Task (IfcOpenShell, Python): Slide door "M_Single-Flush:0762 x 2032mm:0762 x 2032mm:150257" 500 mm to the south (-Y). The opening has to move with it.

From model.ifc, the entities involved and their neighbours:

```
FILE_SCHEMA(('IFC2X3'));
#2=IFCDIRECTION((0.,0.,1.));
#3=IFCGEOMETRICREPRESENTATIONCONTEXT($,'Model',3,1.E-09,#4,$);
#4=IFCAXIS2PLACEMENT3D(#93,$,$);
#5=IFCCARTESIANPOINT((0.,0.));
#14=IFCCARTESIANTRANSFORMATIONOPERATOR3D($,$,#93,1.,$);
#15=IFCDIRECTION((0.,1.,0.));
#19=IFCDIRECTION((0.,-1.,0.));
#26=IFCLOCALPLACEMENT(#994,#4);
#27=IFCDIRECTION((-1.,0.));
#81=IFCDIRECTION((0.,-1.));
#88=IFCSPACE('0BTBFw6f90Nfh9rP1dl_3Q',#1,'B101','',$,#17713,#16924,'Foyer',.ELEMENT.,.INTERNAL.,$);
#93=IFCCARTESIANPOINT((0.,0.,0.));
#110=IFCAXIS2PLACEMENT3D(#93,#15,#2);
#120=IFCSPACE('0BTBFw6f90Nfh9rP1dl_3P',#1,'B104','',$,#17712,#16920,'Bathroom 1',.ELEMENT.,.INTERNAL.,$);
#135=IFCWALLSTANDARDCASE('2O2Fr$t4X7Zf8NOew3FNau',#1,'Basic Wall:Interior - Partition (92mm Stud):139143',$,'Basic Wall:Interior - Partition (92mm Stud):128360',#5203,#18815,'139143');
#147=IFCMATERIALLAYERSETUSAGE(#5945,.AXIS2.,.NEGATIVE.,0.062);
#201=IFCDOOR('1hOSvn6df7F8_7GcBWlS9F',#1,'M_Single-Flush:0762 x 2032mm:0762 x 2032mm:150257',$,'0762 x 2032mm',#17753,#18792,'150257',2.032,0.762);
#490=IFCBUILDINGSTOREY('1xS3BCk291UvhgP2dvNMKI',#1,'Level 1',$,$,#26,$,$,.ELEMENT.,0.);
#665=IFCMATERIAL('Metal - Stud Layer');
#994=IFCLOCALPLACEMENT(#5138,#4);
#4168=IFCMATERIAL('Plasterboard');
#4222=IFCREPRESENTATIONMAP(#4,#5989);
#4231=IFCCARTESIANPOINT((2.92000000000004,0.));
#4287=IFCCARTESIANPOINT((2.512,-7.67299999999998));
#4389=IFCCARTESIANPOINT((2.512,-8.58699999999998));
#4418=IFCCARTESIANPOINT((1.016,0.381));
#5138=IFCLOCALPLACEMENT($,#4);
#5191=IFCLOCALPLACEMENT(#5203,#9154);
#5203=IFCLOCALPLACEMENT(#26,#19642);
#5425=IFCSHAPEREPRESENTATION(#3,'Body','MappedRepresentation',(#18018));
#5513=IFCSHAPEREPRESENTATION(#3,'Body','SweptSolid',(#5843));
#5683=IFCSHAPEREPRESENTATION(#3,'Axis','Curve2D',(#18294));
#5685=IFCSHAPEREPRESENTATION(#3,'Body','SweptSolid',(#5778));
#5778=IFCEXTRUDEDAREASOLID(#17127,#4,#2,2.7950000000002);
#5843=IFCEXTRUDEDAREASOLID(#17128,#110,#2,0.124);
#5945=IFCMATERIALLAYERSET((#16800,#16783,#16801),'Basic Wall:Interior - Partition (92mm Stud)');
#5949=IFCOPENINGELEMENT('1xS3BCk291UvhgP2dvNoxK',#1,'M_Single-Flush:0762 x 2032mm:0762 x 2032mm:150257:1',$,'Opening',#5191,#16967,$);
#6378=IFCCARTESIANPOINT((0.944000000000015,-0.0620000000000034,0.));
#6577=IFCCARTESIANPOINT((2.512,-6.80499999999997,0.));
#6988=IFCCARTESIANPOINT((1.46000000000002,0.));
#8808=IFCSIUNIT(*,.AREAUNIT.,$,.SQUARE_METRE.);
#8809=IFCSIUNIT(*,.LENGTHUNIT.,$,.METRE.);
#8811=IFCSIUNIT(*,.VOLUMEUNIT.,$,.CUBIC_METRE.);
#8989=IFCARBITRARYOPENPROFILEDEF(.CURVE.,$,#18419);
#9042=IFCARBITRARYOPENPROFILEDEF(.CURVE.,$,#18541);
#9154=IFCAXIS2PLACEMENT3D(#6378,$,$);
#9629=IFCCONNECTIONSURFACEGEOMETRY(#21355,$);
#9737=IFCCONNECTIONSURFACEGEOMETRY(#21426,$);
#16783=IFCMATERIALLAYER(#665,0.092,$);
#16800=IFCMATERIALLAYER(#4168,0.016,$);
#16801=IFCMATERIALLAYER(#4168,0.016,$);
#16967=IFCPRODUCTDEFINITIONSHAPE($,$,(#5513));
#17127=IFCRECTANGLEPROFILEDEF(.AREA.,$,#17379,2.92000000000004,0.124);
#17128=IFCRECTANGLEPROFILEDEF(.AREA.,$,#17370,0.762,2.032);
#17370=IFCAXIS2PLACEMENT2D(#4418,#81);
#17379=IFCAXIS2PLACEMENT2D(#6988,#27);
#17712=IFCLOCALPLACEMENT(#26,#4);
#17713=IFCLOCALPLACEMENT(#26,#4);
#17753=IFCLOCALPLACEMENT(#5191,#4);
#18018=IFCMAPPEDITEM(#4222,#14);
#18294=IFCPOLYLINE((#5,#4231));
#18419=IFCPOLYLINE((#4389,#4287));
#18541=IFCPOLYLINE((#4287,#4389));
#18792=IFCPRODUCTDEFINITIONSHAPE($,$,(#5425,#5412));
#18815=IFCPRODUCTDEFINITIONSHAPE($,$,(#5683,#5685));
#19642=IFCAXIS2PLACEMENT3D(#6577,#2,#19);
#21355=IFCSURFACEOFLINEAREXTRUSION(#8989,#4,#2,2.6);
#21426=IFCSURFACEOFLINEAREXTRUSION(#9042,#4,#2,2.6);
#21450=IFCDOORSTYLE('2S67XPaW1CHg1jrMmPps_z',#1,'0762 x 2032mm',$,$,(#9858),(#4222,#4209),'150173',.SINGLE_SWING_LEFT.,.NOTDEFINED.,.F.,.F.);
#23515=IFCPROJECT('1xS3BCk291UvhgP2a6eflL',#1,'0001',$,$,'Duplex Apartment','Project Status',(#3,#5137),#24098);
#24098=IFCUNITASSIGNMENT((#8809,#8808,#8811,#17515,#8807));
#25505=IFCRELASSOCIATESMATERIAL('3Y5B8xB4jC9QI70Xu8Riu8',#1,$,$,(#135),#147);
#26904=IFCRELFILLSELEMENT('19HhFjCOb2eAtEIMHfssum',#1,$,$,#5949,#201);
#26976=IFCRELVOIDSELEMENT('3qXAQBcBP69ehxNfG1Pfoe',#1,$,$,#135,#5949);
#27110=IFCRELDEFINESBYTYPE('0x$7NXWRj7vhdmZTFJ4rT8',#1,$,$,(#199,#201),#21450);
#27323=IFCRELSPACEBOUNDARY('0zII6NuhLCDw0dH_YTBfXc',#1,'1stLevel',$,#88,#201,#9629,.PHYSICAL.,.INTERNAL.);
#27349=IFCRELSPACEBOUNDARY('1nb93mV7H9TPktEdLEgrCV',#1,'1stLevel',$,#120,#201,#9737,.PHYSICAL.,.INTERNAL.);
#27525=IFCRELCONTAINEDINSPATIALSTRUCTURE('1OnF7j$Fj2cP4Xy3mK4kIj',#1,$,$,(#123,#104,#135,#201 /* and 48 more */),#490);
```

```python
import numpy as np
import ifcopenshell
import ifcopenshell.api.geometry
import ifcopenshell.util.placement
import ifcopenshell.util.unit

model = ifcopenshell.open("model.ifc")
unit_scale = ifcopenshell.util.unit.calculate_unit_scale(model)

door = model.by_id(201)
opening = door.FillsVoids[0].RelatingOpeningElement
wall = opening.VoidsElements[0].RelatingBuildingElement

wall_matrix = ifcopenshell.util.placement.get_local_placement(wall.ObjectPlacement)
shift = wall_matrix[:3, 0] * 0.5 / unit_scale
before = ifcopenshell.util.placement.get_local_placement(door.ObjectPlacement)[:3, 3].copy()

# The door is placed relative to its opening, so it follows when the opening moves.
matrix = ifcopenshell.util.placement.get_local_placement(opening.ObjectPlacement)
matrix[:3, 3] += shift
ifcopenshell.api.geometry.edit_object_placement(
    model, product=opening, matrix=matrix, is_si=False, should_transform_children=True
)

# Space boundary surfaces are stored in each space's coordinates; move them too.
for rel in door.ProvidesBoundaries:
    if not rel.ConnectionGeometry:
        continue
    surface = rel.ConnectionGeometry.SurfaceOnRelatingElement
    space_matrix = ifcopenshell.util.placement.get_local_placement(rel.RelatingSpace.ObjectPlacement)
    point = np.array(surface.Position.Location.Coordinates) + space_matrix[:3, :3].T @ shift
    surface.Position = model.createIfcAxis2Placement3D(
        model.createIfcCartesianPoint(point.tolist()), surface.Position.Axis, surface.Position.RefDirection
    )

after = ifcopenshell.util.placement.get_local_placement(door.ObjectPlacement)[:3, 3]
print("door moved by", (after - before).round(3) + 0.0)

model.write("model_v2.ifc")
```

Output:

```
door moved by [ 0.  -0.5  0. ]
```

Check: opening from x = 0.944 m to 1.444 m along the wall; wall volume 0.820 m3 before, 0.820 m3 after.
